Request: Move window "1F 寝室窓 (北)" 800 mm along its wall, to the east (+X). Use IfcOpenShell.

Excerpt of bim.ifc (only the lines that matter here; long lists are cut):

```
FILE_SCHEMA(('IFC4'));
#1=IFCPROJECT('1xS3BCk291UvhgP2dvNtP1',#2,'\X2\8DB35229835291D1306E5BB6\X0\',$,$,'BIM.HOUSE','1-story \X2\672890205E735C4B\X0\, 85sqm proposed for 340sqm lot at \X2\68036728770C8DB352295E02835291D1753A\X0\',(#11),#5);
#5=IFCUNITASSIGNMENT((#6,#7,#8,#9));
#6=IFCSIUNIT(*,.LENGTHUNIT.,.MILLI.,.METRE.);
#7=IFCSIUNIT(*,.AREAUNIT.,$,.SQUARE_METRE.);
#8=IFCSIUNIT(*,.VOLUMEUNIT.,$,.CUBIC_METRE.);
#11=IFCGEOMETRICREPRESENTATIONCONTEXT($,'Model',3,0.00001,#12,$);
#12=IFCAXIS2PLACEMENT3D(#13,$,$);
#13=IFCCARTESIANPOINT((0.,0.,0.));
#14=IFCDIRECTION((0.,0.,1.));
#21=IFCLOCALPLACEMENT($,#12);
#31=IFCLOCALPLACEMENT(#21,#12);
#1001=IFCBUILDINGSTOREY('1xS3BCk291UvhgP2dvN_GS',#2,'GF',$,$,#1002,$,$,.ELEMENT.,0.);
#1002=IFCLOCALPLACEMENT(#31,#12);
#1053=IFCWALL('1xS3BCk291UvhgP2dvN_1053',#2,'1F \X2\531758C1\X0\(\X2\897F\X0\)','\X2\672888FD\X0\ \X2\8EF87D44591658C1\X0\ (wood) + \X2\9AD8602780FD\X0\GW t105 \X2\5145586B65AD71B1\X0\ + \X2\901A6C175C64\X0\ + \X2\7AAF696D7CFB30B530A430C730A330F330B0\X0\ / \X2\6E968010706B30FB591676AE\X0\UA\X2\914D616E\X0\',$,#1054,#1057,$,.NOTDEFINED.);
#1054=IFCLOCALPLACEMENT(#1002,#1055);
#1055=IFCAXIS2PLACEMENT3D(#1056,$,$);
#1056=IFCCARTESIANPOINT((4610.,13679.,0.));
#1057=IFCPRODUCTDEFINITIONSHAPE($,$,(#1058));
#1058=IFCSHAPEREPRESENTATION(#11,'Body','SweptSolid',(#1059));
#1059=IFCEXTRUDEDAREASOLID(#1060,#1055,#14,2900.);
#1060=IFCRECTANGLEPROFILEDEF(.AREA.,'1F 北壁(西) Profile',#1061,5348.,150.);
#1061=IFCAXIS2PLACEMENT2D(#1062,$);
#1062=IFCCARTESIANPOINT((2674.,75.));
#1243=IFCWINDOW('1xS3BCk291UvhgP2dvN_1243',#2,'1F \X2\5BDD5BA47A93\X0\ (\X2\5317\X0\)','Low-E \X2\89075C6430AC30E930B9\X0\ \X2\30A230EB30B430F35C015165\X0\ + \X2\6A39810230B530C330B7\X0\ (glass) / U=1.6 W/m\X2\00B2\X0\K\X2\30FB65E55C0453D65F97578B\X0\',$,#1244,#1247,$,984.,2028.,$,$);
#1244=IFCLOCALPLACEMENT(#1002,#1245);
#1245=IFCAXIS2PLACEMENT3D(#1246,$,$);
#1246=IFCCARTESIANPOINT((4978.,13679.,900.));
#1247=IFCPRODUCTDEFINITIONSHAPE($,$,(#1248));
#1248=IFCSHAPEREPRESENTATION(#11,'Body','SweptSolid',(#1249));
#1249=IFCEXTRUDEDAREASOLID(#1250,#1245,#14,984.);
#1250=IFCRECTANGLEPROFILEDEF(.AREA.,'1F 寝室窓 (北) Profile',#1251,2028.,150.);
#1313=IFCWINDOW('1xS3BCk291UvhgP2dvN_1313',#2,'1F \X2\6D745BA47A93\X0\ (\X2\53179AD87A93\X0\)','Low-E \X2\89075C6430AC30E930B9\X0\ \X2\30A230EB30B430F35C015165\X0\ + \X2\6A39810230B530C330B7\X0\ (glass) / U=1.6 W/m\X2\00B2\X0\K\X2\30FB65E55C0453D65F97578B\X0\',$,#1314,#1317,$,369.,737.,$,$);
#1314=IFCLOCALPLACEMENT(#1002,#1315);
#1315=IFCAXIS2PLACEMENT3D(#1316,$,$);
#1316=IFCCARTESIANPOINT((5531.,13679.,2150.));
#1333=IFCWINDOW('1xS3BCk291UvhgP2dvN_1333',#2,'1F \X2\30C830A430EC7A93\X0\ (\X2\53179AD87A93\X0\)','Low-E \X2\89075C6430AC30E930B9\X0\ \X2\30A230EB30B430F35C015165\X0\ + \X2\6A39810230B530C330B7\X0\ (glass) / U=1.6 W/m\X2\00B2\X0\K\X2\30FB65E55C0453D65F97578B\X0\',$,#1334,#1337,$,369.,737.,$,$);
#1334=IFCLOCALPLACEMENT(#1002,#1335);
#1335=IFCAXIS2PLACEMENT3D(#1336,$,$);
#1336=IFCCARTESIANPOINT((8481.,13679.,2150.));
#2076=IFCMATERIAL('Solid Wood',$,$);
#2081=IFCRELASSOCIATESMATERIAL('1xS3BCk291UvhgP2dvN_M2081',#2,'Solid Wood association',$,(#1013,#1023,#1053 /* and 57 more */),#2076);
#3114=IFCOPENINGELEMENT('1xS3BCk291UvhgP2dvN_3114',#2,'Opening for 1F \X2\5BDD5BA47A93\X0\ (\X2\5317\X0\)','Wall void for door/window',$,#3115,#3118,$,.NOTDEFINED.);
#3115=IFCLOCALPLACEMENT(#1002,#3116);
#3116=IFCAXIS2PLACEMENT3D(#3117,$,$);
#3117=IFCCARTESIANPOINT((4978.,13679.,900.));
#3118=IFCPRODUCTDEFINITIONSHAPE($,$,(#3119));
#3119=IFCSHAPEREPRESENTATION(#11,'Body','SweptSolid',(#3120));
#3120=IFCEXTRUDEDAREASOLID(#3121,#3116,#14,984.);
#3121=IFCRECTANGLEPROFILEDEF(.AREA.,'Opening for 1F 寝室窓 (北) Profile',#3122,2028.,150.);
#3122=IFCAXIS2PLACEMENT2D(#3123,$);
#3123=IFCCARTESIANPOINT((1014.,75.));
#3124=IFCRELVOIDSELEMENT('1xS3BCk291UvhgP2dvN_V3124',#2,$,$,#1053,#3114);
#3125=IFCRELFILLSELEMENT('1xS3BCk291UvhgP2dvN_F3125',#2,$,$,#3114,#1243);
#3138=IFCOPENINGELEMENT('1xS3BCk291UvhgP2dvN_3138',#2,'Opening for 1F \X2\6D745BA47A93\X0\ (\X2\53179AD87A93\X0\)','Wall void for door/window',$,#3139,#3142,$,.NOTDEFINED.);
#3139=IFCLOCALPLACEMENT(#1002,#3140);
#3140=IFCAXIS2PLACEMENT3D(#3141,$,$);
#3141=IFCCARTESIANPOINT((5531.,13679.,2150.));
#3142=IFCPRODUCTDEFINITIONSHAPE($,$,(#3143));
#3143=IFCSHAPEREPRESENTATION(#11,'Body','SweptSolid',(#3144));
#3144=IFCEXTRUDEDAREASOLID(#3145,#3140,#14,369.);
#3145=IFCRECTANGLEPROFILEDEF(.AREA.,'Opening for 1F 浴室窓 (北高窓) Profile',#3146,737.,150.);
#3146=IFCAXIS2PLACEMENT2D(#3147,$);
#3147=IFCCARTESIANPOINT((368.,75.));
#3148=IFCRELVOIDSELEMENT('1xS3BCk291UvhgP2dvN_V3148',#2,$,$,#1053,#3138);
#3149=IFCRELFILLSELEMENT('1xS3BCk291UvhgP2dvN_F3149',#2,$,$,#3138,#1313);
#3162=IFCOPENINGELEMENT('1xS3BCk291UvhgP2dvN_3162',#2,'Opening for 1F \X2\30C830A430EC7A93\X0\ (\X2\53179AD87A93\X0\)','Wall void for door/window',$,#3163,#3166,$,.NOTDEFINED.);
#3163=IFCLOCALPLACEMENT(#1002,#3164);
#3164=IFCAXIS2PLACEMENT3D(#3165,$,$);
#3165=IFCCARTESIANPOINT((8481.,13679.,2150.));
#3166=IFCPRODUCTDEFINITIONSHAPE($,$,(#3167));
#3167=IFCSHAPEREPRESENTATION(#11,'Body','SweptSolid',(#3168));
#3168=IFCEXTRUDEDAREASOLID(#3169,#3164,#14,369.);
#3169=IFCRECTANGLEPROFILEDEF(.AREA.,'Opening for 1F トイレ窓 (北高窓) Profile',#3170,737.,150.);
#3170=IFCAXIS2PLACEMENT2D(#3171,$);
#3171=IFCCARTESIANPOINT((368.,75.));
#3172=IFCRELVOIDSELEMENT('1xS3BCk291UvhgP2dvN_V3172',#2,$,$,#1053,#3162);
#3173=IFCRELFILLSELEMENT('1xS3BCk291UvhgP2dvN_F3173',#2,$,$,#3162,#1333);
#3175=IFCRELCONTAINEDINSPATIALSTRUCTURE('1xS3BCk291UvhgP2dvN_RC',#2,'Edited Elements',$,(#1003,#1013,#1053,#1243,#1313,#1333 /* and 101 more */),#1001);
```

```python
import ifcopenshell
import ifcopenshell.api.geometry
import ifcopenshell.util.placement

model = ifcopenshell.open("bim.ifc")

window = model.by_id(1243)
opening = window.FillsVoids[0].RelatingOpeningElement
wall = opening.VoidsElements[0].RelatingBuildingElement

wall_matrix = ifcopenshell.util.placement.get_local_placement(wall.ObjectPlacement)
shift = wall_matrix[:3, 0] * 800.0
before = ifcopenshell.util.placement.get_local_placement(window.ObjectPlacement)[:3, 3].copy()

# The window is not placed relative to its opening, so move both.
for product in (opening, window):
    matrix = ifcopenshell.util.placement.get_local_placement(product.ObjectPlacement)
    matrix[:3, 3] += shift
    ifcopenshell.api.geometry.edit_object_placement(model, product=product, matrix=matrix, is_si=False)

after = ifcopenshell.util.placement.get_local_placement(window.ObjectPlacement)[:3, 3]
print("window moved by", (after - before).round(3) + 0.0)

model.write("bim_updated.ifc")
```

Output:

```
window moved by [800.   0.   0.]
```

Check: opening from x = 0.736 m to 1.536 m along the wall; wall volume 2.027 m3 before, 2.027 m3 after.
